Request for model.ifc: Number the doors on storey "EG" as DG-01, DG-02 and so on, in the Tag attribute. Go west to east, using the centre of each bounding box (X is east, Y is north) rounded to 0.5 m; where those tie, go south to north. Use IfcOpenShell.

First a look at what the model holds.

```python
import ifcopenshell
import ifcopenshell.util.element
import ifcopenshell.util.placement

model = ifcopenshell.open("model.ifc")
print(model.schema)
storey = next(s for s in model.by_type("IfcBuildingStorey") if s.Name == "EG")
doors = [e for e in ifcopenshell.util.element.get_decomposition(storey) if e.is_a("IfcDoor")]
for e in sorted(doors, key=lambda e: e.id()):
    origin = ifcopenshell.util.placement.get_local_placement(e.ObjectPlacement)[:3, 3]
    print(e.id(), e.Tag, e.Name, origin.round(2) + 0.0, sep=" | ")
```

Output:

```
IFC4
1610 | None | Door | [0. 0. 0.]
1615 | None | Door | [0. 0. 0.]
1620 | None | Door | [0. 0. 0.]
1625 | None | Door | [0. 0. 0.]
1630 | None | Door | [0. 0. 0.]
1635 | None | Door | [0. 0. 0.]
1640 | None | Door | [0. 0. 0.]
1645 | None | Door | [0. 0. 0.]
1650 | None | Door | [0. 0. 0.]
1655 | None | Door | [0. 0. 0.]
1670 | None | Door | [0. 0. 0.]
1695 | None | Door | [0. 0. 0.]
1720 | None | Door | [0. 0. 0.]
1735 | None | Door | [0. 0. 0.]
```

```python
import ifcopenshell
import ifcopenshell.geom
import ifcopenshell.util.element
import ifcopenshell.util.shape

model = ifcopenshell.open("model.ifc")
settings = ifcopenshell.geom.settings()
settings.set("use-world-coords", True)


def centre(element):
    shape = ifcopenshell.geom.create_shape(settings, element)
    return ifcopenshell.util.shape.get_bbox_centroid(shape.geometry)


storey = next(s for s in model.by_type("IfcBuildingStorey") if s.Name == "EG")
doors = [e for e in ifcopenshell.util.element.get_decomposition(storey) if e.is_a("IfcDoor")]

# Insertion points can sit at a corner or the storey origin, so sort by the geometry (in metres).
centres = {e: centre(e) for e in doors}
doors.sort(key=lambda e: (round(centres[e][0] / 0.5), centres[e][1]))

for i, e in enumerate(doors, start=1):
    number = f"DG-{i:02d}"
    e.Tag = number
    print(e.id(), number)

model.write("model_edited.ifc")
```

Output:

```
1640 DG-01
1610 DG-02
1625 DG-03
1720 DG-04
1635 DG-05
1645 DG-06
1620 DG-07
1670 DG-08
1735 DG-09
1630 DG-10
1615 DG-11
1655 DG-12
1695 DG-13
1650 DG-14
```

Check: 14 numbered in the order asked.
